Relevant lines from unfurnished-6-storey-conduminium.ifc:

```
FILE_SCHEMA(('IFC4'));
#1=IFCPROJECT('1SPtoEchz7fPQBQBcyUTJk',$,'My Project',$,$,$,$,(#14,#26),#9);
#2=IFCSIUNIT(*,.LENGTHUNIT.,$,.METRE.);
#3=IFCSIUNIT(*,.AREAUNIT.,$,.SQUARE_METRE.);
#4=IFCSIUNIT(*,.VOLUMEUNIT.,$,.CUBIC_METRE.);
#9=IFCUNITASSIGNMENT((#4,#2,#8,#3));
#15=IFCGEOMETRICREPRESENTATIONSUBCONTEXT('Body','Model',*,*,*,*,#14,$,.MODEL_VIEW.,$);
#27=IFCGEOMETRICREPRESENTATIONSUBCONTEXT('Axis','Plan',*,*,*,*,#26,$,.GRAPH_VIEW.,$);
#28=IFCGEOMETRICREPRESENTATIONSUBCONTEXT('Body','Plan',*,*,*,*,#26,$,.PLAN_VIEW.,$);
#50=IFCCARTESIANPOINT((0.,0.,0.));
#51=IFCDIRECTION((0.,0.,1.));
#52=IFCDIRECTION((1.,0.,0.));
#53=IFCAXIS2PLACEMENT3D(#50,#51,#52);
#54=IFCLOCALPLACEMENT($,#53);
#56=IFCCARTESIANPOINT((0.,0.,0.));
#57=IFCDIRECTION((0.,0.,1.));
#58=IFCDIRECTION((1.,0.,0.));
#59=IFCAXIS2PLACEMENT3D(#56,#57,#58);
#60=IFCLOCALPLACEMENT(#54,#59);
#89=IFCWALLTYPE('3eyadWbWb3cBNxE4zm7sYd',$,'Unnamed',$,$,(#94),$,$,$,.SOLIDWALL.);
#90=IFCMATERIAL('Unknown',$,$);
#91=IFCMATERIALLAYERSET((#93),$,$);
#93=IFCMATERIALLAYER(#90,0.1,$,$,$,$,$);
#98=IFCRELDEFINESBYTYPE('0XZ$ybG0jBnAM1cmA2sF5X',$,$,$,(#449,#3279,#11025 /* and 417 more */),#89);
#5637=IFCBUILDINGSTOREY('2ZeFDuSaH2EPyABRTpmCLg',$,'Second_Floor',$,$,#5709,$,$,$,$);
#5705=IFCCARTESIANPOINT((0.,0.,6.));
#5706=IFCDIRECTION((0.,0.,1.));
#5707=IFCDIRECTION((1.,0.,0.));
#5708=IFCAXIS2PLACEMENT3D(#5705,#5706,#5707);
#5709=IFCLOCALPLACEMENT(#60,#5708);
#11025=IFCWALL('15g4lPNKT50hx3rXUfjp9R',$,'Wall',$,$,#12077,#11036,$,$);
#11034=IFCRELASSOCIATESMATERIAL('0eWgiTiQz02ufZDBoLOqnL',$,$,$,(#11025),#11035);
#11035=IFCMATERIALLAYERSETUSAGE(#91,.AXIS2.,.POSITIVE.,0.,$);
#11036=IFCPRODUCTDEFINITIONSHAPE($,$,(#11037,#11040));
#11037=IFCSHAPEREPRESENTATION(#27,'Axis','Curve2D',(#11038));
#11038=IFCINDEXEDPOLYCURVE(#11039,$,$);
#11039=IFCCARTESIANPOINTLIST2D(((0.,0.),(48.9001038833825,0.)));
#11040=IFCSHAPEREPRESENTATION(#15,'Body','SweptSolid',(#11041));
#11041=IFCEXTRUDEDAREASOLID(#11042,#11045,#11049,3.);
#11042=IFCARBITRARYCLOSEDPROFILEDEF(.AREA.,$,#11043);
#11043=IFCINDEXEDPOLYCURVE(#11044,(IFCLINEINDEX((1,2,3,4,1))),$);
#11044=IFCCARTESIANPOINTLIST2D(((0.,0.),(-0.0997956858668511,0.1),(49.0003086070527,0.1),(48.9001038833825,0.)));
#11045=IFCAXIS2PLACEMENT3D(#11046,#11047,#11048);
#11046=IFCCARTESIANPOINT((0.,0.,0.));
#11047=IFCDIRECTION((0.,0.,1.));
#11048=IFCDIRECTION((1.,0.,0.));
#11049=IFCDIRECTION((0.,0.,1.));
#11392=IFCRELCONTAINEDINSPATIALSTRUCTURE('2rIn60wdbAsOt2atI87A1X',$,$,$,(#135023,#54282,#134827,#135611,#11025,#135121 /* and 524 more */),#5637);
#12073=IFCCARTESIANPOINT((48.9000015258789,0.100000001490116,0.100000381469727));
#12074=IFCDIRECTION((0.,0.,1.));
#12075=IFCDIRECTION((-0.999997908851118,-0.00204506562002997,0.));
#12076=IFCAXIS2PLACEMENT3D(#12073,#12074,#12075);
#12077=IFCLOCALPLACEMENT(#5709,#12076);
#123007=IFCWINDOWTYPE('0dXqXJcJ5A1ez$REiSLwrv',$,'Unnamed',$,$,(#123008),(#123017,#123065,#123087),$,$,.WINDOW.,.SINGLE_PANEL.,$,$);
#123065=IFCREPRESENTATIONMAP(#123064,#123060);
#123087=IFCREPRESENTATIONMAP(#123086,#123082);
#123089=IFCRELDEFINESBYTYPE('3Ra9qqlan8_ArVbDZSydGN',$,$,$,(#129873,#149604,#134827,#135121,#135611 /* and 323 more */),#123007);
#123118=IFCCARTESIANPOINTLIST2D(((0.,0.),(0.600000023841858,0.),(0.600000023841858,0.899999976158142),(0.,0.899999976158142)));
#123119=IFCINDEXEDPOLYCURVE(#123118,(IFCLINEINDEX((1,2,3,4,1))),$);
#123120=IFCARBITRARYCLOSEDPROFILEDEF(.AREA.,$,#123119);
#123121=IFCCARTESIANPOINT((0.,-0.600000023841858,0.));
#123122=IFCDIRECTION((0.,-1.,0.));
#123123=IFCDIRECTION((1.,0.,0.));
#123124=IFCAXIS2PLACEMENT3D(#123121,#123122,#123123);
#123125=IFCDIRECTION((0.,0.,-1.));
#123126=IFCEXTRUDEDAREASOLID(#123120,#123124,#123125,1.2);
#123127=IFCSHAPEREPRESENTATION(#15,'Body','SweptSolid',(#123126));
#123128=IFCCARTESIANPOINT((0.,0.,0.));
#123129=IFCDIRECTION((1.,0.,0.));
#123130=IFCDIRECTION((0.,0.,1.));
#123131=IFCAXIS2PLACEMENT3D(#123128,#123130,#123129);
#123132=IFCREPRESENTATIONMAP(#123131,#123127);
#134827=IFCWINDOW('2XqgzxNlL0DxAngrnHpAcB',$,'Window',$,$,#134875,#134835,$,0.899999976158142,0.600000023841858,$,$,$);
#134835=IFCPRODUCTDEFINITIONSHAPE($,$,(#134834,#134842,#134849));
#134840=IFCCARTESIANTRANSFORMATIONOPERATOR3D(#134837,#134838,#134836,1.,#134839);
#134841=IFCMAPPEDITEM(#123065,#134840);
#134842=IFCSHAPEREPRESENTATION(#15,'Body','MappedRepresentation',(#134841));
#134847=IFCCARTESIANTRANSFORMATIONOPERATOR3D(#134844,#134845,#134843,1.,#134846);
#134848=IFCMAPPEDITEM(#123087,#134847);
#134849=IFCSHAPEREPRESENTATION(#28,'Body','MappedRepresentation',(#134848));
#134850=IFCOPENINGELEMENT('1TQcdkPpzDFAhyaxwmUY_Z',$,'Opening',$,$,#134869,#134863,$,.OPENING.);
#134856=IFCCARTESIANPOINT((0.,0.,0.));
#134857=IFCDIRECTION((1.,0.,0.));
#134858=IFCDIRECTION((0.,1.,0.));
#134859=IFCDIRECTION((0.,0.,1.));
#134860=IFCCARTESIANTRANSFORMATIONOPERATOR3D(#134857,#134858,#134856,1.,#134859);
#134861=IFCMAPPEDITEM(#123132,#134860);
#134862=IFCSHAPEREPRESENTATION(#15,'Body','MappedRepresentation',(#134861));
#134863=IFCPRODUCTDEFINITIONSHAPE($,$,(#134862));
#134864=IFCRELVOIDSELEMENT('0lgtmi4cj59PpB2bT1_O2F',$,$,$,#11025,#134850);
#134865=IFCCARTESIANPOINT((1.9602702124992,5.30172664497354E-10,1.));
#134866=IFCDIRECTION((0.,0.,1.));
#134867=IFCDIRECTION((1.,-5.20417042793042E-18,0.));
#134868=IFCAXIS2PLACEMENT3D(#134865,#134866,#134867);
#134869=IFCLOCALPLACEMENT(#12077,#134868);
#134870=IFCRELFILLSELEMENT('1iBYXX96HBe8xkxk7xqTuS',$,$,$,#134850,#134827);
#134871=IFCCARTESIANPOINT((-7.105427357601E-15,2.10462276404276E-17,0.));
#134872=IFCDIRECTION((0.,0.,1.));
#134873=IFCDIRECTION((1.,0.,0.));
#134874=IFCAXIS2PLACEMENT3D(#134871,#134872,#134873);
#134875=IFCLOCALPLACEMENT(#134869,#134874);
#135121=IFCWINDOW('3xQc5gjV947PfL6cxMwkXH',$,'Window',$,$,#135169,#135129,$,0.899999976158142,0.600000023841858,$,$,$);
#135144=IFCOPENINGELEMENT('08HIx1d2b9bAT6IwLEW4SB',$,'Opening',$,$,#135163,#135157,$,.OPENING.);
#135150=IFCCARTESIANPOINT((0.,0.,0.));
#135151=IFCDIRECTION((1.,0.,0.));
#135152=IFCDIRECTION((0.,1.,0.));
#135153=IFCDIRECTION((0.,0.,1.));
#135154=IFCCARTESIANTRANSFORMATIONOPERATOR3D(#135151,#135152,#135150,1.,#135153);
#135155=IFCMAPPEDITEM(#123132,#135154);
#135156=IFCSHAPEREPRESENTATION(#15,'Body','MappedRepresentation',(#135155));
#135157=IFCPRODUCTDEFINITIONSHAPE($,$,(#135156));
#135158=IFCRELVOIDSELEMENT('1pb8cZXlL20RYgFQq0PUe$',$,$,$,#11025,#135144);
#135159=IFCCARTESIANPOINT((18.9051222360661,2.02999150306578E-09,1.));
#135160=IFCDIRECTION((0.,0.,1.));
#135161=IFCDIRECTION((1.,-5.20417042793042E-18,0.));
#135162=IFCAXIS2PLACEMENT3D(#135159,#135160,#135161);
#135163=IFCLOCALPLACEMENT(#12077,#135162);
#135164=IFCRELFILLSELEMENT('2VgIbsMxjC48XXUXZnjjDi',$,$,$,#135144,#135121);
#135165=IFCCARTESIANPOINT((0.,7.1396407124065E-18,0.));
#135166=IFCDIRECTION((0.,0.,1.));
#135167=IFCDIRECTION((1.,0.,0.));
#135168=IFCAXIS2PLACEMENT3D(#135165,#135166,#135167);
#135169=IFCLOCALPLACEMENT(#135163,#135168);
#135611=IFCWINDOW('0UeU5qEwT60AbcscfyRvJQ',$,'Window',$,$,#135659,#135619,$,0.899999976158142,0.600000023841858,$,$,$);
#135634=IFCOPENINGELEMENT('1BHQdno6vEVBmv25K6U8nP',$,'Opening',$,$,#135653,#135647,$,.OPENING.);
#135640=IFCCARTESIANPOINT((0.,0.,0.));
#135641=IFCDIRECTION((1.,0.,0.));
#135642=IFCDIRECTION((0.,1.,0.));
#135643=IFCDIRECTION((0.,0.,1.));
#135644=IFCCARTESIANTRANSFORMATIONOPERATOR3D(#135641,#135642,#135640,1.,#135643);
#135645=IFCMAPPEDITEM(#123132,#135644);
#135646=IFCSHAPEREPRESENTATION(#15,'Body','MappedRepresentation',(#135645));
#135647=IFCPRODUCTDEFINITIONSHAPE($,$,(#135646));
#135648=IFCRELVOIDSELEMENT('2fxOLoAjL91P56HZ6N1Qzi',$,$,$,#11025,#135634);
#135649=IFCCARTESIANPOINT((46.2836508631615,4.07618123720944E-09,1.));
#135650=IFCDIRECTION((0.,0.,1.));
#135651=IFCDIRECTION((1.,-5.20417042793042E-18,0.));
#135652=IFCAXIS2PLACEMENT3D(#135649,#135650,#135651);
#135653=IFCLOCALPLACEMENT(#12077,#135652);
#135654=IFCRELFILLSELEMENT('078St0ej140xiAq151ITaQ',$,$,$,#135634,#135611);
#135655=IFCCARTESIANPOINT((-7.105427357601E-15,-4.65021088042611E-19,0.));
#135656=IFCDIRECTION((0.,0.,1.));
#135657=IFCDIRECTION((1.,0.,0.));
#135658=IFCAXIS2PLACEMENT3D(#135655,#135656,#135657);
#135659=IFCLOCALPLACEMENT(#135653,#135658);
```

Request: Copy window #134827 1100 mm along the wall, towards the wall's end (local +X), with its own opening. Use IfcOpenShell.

```python
import ifcopenshell
import ifcopenshell.api.feature
import ifcopenshell.api.geometry
import ifcopenshell.api.root
import ifcopenshell.geom
import ifcopenshell.util.element
import ifcopenshell.util.placement
import ifcopenshell.util.shape
import ifcopenshell.util.unit

model = ifcopenshell.open("unfurnished-6-storey-conduminium.ifc")
unit_scale = ifcopenshell.util.unit.calculate_unit_scale(model)
settings = ifcopenshell.geom.settings()


def volume(element):
    """Net volume in cubic metres, openings subtracted."""
    shape = ifcopenshell.geom.create_shape(settings, element)
    return ifcopenshell.util.shape.get_volume(shape.geometry)


window = model.by_guid("2XqgzxNlL0DxAngrnHpAcB")
opening = window.FillsVoids[0].RelatingOpeningElement
wall = opening.VoidsElements[0].RelatingBuildingElement
before = volume(wall)
shift = ifcopenshell.util.placement.get_local_placement(wall.ObjectPlacement)[:3, 0] * 1.1 / unit_scale

# copy_class copies the void relationship, type, container and properties, but no geometry.
new_opening = ifcopenshell.api.root.copy_class(model, product=opening)
new_opening.Representation = ifcopenshell.util.element.copy_deep(
    model, opening.Representation, exclude=["IfcGeometricRepresentationContext", "IfcRepresentationMap"]
)
new_window = ifcopenshell.api.root.copy_class(model, product=window)
new_window.Representation = ifcopenshell.util.element.copy_deep(
    model, window.Representation, exclude=["IfcGeometricRepresentationContext", "IfcRepresentationMap"]
)
ifcopenshell.api.feature.add_filling(model, opening=new_opening, element=new_window)

for old, new in ((opening, new_opening), (window, new_window)):
    matrix = ifcopenshell.util.placement.get_local_placement(old.ObjectPlacement)
    matrix[:3, 3] += shift
    ifcopenshell.api.geometry.edit_object_placement(model, product=new, matrix=matrix, is_si=False)

after = volume(wall)

print(f"wall volume {before:.3f} -> {after:.3f} m3")

model.write("unfurnished-6-storey-conduminium_v2.ifc")
```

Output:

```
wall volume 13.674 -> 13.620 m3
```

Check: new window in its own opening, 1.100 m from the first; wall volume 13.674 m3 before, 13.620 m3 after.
